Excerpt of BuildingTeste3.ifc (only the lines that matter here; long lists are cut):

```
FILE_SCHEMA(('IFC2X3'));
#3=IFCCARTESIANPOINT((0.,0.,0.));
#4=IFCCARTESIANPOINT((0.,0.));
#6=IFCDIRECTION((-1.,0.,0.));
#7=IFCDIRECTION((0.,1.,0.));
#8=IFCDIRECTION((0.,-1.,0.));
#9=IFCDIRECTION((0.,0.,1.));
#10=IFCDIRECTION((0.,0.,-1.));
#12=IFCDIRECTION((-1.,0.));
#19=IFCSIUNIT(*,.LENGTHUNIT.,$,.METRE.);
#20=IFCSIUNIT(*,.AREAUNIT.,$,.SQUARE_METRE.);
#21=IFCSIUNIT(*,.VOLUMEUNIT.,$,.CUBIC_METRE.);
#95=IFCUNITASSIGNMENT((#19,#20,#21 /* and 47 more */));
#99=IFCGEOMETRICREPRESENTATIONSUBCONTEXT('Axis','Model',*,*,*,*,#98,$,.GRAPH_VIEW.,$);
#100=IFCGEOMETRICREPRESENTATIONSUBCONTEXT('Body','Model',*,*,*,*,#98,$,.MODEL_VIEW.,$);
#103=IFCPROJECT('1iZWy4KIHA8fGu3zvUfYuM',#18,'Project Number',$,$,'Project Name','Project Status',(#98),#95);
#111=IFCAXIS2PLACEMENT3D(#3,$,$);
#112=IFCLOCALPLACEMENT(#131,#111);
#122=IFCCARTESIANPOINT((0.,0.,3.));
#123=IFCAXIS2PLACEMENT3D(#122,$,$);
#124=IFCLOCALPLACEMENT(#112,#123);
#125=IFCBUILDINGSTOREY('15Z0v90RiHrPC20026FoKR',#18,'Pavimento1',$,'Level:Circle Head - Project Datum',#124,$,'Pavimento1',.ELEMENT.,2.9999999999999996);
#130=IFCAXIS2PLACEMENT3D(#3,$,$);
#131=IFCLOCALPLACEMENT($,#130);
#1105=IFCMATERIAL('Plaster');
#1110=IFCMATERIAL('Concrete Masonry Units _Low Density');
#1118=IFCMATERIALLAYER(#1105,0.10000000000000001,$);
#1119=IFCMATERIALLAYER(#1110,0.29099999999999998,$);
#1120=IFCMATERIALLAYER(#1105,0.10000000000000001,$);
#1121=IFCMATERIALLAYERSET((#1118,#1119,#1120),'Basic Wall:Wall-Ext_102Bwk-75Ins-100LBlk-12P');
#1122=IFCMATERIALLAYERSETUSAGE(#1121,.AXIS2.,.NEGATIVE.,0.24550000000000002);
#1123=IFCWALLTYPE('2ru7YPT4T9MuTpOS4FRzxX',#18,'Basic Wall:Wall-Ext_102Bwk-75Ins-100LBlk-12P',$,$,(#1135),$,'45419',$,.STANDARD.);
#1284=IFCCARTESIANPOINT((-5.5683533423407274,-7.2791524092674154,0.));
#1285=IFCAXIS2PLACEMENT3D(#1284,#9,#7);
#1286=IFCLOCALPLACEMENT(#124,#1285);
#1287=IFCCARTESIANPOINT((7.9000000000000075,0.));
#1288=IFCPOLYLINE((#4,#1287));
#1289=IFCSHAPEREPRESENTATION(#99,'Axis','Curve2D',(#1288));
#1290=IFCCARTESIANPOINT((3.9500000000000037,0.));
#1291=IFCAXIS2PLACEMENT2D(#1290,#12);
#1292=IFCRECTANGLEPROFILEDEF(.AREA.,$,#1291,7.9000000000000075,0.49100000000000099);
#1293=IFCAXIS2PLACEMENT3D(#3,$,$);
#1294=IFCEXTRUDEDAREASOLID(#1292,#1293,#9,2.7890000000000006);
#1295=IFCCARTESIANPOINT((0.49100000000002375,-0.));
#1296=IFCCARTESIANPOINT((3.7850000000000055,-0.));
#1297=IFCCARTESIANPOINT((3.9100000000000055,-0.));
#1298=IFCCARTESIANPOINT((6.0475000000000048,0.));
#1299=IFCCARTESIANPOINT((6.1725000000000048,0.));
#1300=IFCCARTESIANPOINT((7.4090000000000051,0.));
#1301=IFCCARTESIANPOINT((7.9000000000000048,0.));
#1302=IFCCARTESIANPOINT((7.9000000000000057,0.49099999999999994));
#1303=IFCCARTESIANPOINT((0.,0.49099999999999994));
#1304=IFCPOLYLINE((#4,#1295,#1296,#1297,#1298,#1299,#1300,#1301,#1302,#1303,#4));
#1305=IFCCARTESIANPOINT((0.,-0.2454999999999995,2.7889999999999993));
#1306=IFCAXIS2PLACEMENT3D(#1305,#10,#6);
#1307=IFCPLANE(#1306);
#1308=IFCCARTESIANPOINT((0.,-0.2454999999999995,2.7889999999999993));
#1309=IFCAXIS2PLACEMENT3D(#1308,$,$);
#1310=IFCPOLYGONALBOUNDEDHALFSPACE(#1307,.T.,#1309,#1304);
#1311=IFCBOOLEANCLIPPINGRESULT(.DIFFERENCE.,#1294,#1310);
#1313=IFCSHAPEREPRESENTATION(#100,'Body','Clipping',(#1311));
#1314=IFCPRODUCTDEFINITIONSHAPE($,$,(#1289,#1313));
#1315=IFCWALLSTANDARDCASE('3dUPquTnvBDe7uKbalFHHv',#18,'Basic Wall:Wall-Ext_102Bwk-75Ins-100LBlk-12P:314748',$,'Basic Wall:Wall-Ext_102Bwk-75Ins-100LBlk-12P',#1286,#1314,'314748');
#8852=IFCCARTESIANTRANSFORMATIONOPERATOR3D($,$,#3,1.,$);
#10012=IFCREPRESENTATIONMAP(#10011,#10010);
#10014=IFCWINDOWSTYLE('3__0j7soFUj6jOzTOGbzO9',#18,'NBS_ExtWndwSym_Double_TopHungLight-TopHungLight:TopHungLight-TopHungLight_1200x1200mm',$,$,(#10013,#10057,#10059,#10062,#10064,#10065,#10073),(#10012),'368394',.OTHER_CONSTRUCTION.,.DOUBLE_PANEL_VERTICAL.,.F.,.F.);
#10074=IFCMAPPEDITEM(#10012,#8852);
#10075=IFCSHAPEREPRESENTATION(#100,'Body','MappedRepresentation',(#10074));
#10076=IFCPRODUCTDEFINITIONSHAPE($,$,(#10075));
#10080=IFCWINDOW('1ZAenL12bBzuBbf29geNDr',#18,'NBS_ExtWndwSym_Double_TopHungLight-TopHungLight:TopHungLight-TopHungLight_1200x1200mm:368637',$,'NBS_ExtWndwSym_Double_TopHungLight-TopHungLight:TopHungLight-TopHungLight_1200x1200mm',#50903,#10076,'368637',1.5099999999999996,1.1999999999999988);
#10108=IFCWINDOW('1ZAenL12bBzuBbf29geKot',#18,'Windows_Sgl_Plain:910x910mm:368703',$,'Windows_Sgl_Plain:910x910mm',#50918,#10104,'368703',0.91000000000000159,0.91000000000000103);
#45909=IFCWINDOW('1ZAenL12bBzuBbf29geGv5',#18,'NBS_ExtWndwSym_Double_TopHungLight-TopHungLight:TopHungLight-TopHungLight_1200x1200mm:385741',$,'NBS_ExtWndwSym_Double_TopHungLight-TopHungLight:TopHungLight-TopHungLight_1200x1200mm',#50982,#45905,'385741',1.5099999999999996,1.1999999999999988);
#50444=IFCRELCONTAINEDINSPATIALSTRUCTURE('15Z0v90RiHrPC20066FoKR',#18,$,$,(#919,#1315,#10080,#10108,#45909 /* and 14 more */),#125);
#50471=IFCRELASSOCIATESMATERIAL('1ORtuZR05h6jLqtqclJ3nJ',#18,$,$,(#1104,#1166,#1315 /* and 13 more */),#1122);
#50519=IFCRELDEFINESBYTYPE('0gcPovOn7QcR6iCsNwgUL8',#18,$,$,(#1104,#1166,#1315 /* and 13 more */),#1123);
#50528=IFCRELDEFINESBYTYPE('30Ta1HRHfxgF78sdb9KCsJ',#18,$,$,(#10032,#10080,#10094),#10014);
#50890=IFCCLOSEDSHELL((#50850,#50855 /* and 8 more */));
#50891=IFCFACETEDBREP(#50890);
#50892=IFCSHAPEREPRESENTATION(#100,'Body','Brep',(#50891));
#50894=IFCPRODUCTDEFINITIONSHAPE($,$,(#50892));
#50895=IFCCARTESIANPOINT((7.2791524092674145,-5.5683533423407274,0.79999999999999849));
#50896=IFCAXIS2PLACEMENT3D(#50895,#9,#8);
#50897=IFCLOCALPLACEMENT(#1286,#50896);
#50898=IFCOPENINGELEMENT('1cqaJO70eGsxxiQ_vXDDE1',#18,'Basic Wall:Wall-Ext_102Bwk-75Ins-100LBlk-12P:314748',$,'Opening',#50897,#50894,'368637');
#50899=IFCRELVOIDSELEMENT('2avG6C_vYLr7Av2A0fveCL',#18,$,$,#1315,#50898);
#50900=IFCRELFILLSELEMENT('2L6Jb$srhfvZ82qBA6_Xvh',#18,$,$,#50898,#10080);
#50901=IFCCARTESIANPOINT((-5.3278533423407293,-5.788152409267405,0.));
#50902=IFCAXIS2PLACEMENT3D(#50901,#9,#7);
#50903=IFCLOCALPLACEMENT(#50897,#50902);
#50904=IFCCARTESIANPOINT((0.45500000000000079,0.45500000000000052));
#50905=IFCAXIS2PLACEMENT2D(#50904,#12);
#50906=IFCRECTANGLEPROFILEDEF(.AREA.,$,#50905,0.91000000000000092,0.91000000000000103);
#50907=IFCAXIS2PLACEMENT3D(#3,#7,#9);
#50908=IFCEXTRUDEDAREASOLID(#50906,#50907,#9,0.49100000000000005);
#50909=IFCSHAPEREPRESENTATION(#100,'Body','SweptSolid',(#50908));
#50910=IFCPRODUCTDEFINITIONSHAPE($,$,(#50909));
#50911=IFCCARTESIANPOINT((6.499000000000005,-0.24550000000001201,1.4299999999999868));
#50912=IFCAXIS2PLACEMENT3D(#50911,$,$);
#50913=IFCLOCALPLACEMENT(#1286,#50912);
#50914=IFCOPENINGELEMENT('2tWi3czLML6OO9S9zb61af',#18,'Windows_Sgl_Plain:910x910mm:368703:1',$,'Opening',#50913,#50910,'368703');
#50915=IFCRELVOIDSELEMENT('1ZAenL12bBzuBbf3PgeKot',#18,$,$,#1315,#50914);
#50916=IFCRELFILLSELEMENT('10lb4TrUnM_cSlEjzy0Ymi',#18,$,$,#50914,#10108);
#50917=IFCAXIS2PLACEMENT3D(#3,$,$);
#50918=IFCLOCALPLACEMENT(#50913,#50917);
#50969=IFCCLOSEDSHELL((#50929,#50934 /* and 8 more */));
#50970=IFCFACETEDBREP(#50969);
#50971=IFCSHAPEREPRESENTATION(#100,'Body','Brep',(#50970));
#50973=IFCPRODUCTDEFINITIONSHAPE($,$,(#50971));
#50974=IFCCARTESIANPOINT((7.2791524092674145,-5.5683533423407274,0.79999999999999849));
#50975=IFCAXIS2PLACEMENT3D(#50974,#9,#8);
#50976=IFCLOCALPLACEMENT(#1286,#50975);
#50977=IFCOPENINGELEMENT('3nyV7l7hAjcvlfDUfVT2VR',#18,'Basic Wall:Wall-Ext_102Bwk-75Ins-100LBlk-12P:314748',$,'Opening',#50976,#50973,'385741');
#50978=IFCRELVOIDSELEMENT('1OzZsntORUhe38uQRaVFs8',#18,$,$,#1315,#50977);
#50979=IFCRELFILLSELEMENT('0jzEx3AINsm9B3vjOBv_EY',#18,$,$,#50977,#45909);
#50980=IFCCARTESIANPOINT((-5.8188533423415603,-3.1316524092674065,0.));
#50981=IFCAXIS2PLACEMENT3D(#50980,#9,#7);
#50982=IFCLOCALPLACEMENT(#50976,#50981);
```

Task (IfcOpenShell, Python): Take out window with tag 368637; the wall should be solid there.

```python
import ifcopenshell
import ifcopenshell.api.feature
import ifcopenshell.api.root
import ifcopenshell.geom
import ifcopenshell.util.shape

model = ifcopenshell.open("BuildingTeste3.ifc")
settings = ifcopenshell.geom.settings()


def volume(element):
    """Net volume in cubic metres, openings subtracted."""
    shape = ifcopenshell.geom.create_shape(settings, element)
    return ifcopenshell.util.shape.get_volume(shape.geometry)


window = model.by_guid("1ZAenL12bBzuBbf29geNDr")
opening = window.FillsVoids[0].RelatingOpeningElement
wall = opening.VoidsElements[0].RelatingBuildingElement
before = volume(wall)

ifcopenshell.api.root.remove_product(model, product=window)
ifcopenshell.api.feature.remove_feature(model, feature=opening)

after = volume(wall)

print(f"wall volume {before:.3f} -> {after:.3f} m3")

model.write("BuildingTeste3_rev.ifc")
```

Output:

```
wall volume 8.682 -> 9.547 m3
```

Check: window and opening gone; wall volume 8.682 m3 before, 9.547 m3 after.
